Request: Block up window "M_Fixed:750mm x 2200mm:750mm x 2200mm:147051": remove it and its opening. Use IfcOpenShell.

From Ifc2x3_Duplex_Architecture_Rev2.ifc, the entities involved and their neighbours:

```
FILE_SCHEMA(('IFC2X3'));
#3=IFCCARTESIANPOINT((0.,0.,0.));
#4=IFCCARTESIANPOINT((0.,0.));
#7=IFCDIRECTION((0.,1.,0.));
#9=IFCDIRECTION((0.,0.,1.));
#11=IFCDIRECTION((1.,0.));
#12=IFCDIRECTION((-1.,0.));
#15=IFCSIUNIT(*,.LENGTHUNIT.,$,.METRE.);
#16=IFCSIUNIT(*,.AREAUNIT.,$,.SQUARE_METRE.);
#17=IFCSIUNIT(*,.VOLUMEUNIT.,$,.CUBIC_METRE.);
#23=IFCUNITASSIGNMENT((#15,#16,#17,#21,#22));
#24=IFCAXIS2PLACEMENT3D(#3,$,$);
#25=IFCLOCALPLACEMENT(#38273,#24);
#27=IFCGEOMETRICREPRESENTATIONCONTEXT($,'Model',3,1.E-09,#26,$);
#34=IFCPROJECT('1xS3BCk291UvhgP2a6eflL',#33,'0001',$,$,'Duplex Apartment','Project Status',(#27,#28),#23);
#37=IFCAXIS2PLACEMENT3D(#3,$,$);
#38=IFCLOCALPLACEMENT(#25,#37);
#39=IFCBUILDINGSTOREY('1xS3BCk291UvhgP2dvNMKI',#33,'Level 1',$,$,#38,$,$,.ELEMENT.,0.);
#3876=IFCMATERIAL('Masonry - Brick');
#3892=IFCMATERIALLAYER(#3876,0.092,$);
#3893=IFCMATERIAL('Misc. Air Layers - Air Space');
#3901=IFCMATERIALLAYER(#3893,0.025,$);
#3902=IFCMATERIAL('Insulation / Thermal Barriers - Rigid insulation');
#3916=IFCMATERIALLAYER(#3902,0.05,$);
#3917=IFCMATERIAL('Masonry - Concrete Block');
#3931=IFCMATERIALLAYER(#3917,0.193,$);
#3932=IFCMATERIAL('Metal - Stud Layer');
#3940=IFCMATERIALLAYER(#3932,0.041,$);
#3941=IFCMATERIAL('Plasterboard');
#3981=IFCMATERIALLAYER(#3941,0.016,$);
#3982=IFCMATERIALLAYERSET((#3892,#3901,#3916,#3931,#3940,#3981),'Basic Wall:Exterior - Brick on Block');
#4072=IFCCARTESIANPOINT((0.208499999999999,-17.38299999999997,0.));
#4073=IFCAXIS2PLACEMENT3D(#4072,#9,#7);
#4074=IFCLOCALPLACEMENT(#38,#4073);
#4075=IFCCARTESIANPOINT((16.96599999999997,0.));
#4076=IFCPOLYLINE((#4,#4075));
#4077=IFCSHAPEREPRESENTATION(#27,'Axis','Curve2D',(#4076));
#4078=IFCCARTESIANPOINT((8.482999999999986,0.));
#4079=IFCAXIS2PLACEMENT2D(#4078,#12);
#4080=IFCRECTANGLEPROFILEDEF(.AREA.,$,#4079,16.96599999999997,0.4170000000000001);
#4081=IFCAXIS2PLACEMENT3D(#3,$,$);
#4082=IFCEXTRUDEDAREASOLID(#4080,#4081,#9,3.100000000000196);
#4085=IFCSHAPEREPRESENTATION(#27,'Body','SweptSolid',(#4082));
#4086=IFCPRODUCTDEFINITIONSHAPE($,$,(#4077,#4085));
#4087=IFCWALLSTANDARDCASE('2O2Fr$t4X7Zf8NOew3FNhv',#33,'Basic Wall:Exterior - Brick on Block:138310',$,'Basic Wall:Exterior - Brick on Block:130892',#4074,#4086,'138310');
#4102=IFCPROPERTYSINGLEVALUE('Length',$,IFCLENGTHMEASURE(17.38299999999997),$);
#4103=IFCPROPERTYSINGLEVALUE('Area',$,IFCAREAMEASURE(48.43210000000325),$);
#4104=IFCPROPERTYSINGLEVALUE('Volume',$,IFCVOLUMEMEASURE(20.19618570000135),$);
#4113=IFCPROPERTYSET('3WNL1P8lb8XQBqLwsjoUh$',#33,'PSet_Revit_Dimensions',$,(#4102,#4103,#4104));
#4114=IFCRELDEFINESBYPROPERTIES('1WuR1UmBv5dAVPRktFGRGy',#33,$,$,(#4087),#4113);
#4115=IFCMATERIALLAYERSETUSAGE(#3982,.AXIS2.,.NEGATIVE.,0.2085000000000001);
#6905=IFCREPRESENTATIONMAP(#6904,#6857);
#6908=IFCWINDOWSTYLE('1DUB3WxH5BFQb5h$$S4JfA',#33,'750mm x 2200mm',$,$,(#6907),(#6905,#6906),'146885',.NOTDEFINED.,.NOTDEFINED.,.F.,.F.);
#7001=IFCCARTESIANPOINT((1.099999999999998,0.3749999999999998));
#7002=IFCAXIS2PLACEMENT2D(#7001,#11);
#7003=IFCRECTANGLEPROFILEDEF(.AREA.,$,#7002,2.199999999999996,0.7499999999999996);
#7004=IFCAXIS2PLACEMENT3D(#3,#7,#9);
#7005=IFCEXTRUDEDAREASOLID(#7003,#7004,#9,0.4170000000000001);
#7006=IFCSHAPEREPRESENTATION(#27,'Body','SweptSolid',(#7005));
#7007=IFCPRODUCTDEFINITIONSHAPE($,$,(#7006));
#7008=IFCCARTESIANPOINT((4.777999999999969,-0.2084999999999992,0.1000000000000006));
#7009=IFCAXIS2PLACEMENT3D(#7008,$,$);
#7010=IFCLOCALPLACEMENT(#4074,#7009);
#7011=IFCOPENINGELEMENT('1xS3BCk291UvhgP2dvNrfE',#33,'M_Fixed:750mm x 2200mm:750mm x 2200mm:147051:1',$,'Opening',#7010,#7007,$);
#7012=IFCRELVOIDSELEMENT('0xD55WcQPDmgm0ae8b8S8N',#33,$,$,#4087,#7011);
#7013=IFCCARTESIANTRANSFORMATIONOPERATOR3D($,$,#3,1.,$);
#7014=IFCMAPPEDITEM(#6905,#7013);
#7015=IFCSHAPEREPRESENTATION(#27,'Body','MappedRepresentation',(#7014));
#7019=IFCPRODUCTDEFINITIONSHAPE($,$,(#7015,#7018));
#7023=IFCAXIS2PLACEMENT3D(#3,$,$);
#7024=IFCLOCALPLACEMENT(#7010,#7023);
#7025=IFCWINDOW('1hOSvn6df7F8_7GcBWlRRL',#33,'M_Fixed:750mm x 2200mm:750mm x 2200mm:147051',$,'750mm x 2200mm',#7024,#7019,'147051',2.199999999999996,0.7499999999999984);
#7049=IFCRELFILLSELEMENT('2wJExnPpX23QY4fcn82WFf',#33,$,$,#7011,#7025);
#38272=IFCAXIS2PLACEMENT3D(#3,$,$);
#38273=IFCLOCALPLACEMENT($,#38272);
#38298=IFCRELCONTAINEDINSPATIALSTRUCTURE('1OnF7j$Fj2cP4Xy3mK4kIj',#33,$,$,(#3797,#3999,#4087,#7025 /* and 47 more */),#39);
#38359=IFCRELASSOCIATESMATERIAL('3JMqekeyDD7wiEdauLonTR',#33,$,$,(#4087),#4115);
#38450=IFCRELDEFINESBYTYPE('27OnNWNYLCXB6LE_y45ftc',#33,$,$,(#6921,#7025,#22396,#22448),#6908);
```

```python
import ifcopenshell
import ifcopenshell.api.feature
import ifcopenshell.api.pset
import ifcopenshell.api.root
import ifcopenshell.geom
import ifcopenshell.util.element
import ifcopenshell.util.shape
import ifcopenshell.util.unit

model = ifcopenshell.open("Ifc2x3_Duplex_Architecture_Rev2.ifc")
area_scale = ifcopenshell.util.unit.calculate_unit_scale(model, "AREAUNIT")
volume_scale = ifcopenshell.util.unit.calculate_unit_scale(model, "VOLUMEUNIT")
settings = ifcopenshell.geom.settings()


def volume(element):
    """Net volume in cubic metres, openings subtracted."""
    shape = ifcopenshell.geom.create_shape(settings, element)
    return ifcopenshell.util.shape.get_volume(shape.geometry)


window = model.by_guid("1hOSvn6df7F8_7GcBWlRRL")
opening = window.FillsVoids[0].RelatingOpeningElement
wall = opening.VoidsElements[0].RelatingBuildingElement
before = volume(wall)

ifcopenshell.api.root.remove_product(model, product=window)
ifcopenshell.api.feature.remove_feature(model, feature=opening)

after = volume(wall)
thickness = 0.417  # wall thickness in metres

# Update the wall's stored quantities.
pset = model.by_id(ifcopenshell.util.element.get_pset(wall, "PSet_Revit_Dimensions", should_inherit=False)["id"])
ifcopenshell.api.pset.edit_pset(model, pset=pset, properties={
    "Area": model.create_entity("IfcAreaMeasure", after / thickness / area_scale),
    "Volume": model.create_entity("IfcVolumeMeasure", after / volume_scale),
})

print(f"wall volume {before:.3f} -> {after:.3f} m3")

model.write("Ifc2x3_Duplex_Architecture_Rev2_edited.ifc")
```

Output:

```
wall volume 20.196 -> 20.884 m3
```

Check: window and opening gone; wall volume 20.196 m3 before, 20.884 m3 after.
